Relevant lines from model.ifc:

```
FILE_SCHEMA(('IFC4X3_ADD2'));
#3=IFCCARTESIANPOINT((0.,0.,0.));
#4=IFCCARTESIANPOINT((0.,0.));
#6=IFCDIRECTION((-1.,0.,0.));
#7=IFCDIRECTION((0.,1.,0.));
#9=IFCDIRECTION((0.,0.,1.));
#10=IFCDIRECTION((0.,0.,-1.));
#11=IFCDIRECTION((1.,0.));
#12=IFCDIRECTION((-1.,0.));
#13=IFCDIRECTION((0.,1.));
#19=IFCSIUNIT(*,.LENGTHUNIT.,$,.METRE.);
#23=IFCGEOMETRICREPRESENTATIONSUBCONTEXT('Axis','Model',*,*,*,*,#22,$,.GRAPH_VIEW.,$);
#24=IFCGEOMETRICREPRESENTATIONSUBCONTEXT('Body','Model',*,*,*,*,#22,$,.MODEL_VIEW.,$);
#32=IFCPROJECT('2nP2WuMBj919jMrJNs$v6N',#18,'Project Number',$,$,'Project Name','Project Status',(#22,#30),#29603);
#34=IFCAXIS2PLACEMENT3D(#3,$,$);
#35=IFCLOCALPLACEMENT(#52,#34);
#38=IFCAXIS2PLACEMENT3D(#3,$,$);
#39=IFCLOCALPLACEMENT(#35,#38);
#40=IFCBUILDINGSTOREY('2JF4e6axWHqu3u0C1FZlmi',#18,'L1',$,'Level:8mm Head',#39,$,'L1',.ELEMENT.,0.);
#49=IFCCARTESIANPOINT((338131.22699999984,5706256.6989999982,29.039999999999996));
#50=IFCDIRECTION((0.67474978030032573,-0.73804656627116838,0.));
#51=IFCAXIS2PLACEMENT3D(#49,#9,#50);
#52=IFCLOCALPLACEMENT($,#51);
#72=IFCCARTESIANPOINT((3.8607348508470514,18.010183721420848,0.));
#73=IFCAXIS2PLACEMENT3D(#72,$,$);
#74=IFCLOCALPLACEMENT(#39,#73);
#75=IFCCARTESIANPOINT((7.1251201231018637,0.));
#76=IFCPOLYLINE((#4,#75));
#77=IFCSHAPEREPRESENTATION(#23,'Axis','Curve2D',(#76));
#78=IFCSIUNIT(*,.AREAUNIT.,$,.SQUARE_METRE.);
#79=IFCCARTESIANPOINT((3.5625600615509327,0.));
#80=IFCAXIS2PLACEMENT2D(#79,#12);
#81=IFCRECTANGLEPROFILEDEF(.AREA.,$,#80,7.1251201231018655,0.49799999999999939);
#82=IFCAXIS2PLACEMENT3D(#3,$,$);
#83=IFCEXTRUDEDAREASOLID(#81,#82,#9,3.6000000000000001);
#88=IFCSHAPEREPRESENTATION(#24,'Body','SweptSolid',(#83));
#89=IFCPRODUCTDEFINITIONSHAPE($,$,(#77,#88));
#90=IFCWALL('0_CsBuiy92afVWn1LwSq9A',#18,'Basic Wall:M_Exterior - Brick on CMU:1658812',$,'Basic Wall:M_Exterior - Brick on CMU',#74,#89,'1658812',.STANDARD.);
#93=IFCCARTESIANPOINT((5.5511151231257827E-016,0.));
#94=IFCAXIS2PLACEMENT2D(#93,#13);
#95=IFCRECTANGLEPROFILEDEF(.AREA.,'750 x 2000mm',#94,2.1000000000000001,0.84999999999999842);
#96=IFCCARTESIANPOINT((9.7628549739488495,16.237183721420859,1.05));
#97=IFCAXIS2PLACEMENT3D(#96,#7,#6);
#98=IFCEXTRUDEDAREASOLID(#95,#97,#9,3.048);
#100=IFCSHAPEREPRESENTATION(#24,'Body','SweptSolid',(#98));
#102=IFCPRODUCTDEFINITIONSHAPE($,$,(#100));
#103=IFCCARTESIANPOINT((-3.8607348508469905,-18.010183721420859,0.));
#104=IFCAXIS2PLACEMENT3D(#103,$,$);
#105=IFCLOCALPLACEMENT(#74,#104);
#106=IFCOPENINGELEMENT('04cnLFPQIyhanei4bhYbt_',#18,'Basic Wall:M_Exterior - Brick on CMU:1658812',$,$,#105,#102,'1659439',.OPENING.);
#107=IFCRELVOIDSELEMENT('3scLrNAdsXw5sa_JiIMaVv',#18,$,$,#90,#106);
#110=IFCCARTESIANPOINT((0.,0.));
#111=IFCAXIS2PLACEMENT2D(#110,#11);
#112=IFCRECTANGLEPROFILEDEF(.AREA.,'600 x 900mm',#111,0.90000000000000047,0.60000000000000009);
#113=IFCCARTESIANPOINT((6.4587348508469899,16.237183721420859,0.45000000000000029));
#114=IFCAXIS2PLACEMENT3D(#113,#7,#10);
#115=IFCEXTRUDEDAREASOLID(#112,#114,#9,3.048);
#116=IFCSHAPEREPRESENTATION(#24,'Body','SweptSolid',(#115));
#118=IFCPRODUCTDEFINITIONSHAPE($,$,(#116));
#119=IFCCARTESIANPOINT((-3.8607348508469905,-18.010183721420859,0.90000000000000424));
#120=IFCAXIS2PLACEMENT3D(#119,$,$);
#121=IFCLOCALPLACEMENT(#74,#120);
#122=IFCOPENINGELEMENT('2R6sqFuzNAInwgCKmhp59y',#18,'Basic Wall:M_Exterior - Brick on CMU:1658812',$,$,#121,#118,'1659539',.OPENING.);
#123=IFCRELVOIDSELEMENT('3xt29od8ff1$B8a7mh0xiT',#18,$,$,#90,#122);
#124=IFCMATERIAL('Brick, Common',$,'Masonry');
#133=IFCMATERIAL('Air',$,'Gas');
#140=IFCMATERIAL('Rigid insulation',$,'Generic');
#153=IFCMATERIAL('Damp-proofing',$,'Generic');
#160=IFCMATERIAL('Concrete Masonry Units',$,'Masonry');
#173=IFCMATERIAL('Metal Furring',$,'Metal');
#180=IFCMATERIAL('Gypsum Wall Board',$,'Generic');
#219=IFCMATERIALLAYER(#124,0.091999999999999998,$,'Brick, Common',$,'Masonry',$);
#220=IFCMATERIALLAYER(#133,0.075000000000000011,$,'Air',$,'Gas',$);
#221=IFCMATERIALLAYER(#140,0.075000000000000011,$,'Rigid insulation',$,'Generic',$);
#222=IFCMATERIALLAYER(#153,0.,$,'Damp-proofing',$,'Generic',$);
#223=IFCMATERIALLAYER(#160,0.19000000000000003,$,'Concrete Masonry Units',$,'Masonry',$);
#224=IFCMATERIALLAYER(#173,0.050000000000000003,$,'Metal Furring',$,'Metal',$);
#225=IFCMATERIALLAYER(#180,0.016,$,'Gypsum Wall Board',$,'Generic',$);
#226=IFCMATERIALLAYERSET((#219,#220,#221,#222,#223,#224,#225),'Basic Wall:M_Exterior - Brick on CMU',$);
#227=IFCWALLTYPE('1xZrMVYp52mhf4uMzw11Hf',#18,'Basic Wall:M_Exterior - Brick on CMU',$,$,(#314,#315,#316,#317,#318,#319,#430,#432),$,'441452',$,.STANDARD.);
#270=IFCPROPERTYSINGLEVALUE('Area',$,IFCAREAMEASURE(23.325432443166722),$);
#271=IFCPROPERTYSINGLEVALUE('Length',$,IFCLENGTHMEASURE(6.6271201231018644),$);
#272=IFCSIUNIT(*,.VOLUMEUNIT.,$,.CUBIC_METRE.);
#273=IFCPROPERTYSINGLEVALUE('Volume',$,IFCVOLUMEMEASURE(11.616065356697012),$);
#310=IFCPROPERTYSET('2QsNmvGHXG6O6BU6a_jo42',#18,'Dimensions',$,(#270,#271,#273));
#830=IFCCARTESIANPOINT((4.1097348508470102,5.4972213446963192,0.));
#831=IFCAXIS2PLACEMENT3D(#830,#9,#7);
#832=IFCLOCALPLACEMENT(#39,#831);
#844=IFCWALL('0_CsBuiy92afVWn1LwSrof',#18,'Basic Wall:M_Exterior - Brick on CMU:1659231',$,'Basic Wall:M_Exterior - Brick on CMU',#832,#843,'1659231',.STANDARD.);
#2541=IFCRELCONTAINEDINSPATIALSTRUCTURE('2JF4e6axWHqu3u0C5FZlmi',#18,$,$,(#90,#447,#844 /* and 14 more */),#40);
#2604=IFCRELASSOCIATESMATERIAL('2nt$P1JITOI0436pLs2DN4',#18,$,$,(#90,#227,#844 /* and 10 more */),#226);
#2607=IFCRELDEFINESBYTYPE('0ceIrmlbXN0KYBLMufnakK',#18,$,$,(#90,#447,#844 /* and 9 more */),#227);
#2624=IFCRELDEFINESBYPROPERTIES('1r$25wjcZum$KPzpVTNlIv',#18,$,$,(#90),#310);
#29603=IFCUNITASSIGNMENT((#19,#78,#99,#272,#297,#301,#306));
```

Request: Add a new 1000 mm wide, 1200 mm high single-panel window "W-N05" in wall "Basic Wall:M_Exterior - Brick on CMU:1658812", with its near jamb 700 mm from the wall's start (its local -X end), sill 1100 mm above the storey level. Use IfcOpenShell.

```python
import numpy as np
import ifcopenshell
import ifcopenshell.api.feature
import ifcopenshell.api.geometry
import ifcopenshell.api.pset
import ifcopenshell.api.root
import ifcopenshell.api.spatial
import ifcopenshell.geom
import ifcopenshell.util.element
import ifcopenshell.util.placement
import ifcopenshell.util.representation
import ifcopenshell.util.shape
import ifcopenshell.util.unit

model = ifcopenshell.open("model.ifc")
unit_scale = ifcopenshell.util.unit.calculate_unit_scale(model)
area_scale = ifcopenshell.util.unit.calculate_unit_scale(model, "AREAUNIT")
volume_scale = ifcopenshell.util.unit.calculate_unit_scale(model, "VOLUMEUNIT")
settings = ifcopenshell.geom.settings()


def volume(element):
    """Net volume in cubic metres, openings subtracted."""
    shape = ifcopenshell.geom.create_shape(settings, element)
    return ifcopenshell.util.shape.get_volume(shape.geometry)


wall = model.by_id(90)
storey = ifcopenshell.util.element.get_container(wall, ifc_class="IfcBuildingStorey")
context = ifcopenshell.util.representation.get_context(model, "Model", "Body", "MODEL_VIEW")
before = volume(wall)

width, height, from_end, sill = 1, 1.2, 0.7, 1.1  # metres

# The wall runs along its own X axis, and the end named is its -X end.
wall_shape = ifcopenshell.geom.create_shape(settings, wall)
x, y, z = ifcopenshell.util.shape.get_vertices(wall_shape.geometry).T
start = x.min() + from_end
face, thickness = float(y.min()), float(y.max() - y.min())
wall_matrix = ifcopenshell.util.placement.get_local_placement(wall.ObjectPlacement)
level = ifcopenshell.util.placement.get_local_placement(storey.ObjectPlacement)[2, 3]


def in_wall(x, y):
    """Placement at x, y metres in the wall's axes, at sill height."""
    matrix = wall_matrix.copy()
    matrix[:, 3] = wall_matrix @ np.array([x / unit_scale, y / unit_scale, 0.0, 1.0])
    matrix[2, 3] = level + sill / unit_scale
    return matrix


# Opening: a box that overshoots both wall faces by 50 mm.
opening = ifcopenshell.api.root.create_entity(model, ifc_class="IfcOpeningElement", predefined_type="OPENING")
box = ifcopenshell.api.geometry.add_wall_representation(
    model, context=context, length=width, height=height, thickness=thickness + 0.1
)
ifcopenshell.api.geometry.assign_representation(model, product=opening, representation=box)
ifcopenshell.api.geometry.edit_object_placement(model, product=opening, matrix=in_wall(start, face - 0.05), is_si=False)
ifcopenshell.api.feature.add_feature(model, feature=opening, element=wall)

window = ifcopenshell.api.root.create_entity(model, ifc_class="IfcWindow", name="W-N05", predefined_type="WINDOW")
window.OverallWidth, window.OverallHeight = width / unit_scale, height / unit_scale
window.PartitioningType = "SINGLE_PANEL"
body = ifcopenshell.api.geometry.add_window_representation(
    model,
    context=context,
    overall_width=window.OverallWidth,
    overall_height=window.OverallHeight,
    partition_type="SINGLE_PANEL",
)
ifcopenshell.api.geometry.assign_representation(model, product=window, representation=body)
ifcopenshell.api.spatial.assign_container(model, products=[window], relating_structure=storey)
ifcopenshell.api.feature.add_filling(model, opening=opening, element=window)

# Centre the window in the wall's thickness.
ifcopenshell.api.geometry.edit_object_placement(model, product=window, matrix=in_wall(start, face), is_si=False)
window_shape = ifcopenshell.geom.create_shape(settings, window)
depth = ifcopenshell.util.shape.get_vertices(window_shape.geometry)[:, 1]
offset = face + thickness / 2 - (depth.min() + depth.max()) / 2
ifcopenshell.api.geometry.edit_object_placement(model, product=window, matrix=in_wall(start, offset), is_si=False)

after = volume(wall)

# Update the wall's stored quantities.
pset = model.by_id(ifcopenshell.util.element.get_pset(wall, "Dimensions", should_inherit=False)["id"])
ifcopenshell.api.pset.edit_pset(model, pset=pset, properties={
    "Area": model.create_entity("IfcAreaMeasure", after / thickness / area_scale),
    "Volume": model.create_entity("IfcVolumeMeasure", after / volume_scale),
})

print(f"wall volume {before:.3f} -> {after:.3f} m3")

model.write("model-out.ifc")
```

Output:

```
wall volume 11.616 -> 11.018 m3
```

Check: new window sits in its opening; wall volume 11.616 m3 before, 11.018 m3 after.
